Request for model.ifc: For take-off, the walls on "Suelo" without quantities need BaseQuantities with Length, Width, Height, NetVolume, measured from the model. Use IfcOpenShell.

First a look at what the model holds.

```python
import ifcopenshell
import ifcopenshell.util.element
import ifcopenshell.util.unit

model = ifcopenshell.open("model.ifc")
print(model.schema)
for unit_type in ("LENGTHUNIT", "AREAUNIT", "VOLUMEUNIT"):
    print(unit_type, ifcopenshell.util.unit.calculate_unit_scale(model, unit_type))
storey = next(s for s in model.by_type("IfcBuildingStorey") if s.Name == "Suelo")
walls = [e for e in ifcopenshell.util.element.get_decomposition(storey) if e.is_a("IfcWall")]
for e in sorted(walls, key=lambda e: e.id()):
    print(e.id(), e.is_a(), e.Name, list(ifcopenshell.util.element.get_psets(e, qtos_only=True)), sep=" | ")
```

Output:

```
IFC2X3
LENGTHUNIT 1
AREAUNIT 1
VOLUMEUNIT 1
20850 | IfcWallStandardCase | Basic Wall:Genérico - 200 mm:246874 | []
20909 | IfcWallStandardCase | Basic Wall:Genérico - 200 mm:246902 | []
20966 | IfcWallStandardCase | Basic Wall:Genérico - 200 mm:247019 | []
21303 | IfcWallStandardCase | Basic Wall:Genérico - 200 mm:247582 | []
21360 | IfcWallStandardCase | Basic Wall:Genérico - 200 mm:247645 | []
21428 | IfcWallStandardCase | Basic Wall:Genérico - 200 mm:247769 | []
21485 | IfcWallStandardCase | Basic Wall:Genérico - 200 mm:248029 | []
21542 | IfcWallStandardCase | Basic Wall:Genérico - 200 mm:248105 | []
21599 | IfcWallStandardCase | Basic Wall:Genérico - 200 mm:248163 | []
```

```python
import ifcopenshell
import ifcopenshell.api.pset
import ifcopenshell.geom
import ifcopenshell.util.element
import ifcopenshell.util.shape
import ifcopenshell.util.unit

model = ifcopenshell.open("model.ifc")
unit_scale = ifcopenshell.util.unit.calculate_unit_scale(model)
volume_scale = ifcopenshell.util.unit.calculate_unit_scale(model, "VOLUMEUNIT")
settings = ifcopenshell.geom.settings()

storey = next(s for s in model.by_type("IfcBuildingStorey") if s.Name == "Suelo")
walls = [e for e in ifcopenshell.util.element.get_decomposition(storey) if e.is_a("IfcWall")]

for e in sorted(walls, key=lambda e: e.id()):
    if ifcopenshell.util.element.get_psets(e, qtos_only=True, should_inherit=False):
        continue
    # Geometry comes back in metres, in the element's own axes.
    shape = ifcopenshell.geom.create_shape(settings, e)
    values = {
        "Length": ifcopenshell.util.shape.get_x(shape.geometry) / unit_scale,
        "Width": ifcopenshell.util.shape.get_y(shape.geometry) / unit_scale,
        "Height": ifcopenshell.util.shape.get_z(shape.geometry) / unit_scale,
        "NetVolume": ifcopenshell.util.shape.get_volume(shape.geometry) / volume_scale,
    }
    qto = ifcopenshell.api.pset.add_qto(model, product=e, name="BaseQuantities")
    ifcopenshell.api.pset.edit_qto(model, qto=qto, properties=values)
    print(e.id(), {k: round(v, 3) for k, v in values.items()})

model.write("model_rev.ifc")
```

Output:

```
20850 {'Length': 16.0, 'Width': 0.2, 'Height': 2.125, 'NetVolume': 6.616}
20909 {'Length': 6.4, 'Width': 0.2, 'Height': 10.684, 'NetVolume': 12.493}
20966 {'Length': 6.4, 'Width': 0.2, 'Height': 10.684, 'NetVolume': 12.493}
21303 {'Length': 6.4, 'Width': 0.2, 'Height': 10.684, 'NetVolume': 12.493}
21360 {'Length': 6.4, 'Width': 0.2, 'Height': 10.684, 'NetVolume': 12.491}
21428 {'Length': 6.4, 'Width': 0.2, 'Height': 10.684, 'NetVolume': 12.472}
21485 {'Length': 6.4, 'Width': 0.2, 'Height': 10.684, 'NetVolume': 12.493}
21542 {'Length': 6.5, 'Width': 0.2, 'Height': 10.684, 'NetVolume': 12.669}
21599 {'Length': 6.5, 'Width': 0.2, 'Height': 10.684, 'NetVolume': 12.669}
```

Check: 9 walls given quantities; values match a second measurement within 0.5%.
